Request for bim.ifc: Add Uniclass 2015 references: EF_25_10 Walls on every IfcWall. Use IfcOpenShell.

First a look at what the model holds.

```python
import ifcopenshell

model = ifcopenshell.open("bim.ifc")
print(model.schema)
print("classifications:", [c.Name for c in model.by_type("IfcClassification")])
for ifc_class in ("IfcDoor", "IfcRoof", "IfcStair", "IfcWall", "IfcWindow"):
    print(ifc_class, len(model.by_type(ifc_class)))
```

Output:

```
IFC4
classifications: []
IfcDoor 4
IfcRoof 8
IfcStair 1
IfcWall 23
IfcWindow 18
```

```python
import ifcopenshell
import ifcopenshell.api.classification

model = ifcopenshell.open("bim.ifc")

system = ifcopenshell.api.classification.add_classification(model, classification="Uniclass 2015")

codes = {
    "IfcWall": ("EF_25_10", "Walls"),
}
for ifc_class, (code, name) in codes.items():
    products = model.by_type(ifc_class)
    ifcopenshell.api.classification.add_reference(
        model, products=products, classification=system, identification=code, name=name
    )
    print(code, len(products))

model.write("bim_edited.ifc")
```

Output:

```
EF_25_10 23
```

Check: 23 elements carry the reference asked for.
